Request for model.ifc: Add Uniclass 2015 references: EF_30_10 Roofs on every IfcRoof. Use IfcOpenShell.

First a look at what the model holds.

```python
import ifcopenshell

model = ifcopenshell.open("model.ifc")
print(model.schema)
print("classifications:", [c.Name for c in model.by_type("IfcClassification")])
for ifc_class in ("IfcDoor", "IfcRoof", "IfcStair", "IfcWall", "IfcWindow"):
    print(ifc_class, len(model.by_type(ifc_class)))
```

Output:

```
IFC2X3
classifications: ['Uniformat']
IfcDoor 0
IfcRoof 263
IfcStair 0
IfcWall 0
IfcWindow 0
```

```python
import ifcopenshell
import ifcopenshell.api.classification

model = ifcopenshell.open("model.ifc")

# IFC2X3 requires Source and Edition and has no link from the project to the system.
system = model.create_entity("IfcClassification", Source="NBS", Edition="2015", Name="Uniclass 2015")

codes = {
    "IfcRoof": ("EF_30_10", "Roofs"),
}
for ifc_class, (code, name) in codes.items():
    products = model.by_type(ifc_class)
    ifcopenshell.api.classification.add_reference(
        model, products=products, classification=system, identification=code, name=name
    )
    print(code, len(products))

model.write("model_updated.ifc")
```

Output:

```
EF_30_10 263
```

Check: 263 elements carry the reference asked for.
